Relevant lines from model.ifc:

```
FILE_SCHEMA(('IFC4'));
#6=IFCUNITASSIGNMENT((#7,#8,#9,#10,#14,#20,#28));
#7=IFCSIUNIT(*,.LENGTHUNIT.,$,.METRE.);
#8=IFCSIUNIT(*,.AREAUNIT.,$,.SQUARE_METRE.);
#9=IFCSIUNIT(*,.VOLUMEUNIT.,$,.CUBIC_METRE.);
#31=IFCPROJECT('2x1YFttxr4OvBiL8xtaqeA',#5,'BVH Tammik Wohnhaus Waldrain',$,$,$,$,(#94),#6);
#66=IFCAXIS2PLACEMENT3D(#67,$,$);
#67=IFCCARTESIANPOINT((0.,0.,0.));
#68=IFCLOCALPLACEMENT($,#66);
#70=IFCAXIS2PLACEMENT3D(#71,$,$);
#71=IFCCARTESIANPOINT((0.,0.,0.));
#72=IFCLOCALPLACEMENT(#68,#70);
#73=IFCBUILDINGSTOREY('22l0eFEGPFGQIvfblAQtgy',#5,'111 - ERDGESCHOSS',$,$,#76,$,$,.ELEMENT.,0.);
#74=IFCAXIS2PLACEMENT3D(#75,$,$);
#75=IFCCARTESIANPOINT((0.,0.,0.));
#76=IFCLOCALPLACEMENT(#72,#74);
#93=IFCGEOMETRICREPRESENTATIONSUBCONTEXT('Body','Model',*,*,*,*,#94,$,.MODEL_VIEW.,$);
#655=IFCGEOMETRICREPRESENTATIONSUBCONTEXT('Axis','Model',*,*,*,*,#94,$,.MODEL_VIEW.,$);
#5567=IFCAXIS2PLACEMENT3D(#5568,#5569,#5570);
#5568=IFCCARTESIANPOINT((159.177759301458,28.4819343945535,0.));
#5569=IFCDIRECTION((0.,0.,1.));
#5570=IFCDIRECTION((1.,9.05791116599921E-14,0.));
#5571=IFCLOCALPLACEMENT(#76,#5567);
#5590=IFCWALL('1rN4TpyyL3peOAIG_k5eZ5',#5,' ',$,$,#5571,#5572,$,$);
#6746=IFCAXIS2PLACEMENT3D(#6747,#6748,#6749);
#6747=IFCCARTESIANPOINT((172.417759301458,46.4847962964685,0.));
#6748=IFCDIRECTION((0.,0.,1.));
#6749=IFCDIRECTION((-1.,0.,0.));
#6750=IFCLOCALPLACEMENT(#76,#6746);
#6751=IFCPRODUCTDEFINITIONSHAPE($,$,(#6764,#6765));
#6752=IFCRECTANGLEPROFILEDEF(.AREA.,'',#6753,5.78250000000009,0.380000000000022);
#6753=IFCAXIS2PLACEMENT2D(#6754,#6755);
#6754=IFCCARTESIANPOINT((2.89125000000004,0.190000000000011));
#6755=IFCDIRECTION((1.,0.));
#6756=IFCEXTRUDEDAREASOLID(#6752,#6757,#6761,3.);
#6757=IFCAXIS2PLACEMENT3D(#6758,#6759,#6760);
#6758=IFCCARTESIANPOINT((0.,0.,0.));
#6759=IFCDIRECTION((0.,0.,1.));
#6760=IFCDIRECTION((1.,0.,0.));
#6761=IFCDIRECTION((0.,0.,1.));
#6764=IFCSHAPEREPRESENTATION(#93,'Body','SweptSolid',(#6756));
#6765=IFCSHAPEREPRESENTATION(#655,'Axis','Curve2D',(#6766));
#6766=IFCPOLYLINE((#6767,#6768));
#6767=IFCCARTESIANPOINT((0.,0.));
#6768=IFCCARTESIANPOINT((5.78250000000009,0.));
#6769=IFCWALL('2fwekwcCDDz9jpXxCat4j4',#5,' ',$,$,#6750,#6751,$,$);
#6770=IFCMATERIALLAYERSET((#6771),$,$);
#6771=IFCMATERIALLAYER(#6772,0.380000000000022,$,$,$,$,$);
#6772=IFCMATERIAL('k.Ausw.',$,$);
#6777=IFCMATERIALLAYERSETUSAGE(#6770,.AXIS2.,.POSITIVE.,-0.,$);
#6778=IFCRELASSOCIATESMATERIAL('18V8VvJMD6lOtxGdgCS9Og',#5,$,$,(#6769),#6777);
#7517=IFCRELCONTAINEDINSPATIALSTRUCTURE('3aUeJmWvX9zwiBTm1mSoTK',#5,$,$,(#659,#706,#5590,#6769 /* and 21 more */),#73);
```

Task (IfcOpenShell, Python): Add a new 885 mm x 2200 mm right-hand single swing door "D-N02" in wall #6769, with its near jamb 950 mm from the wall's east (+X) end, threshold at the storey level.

```python
import numpy as np
import ifcopenshell
import ifcopenshell.api.feature
import ifcopenshell.api.geometry
import ifcopenshell.api.root
import ifcopenshell.api.spatial
import ifcopenshell.geom
import ifcopenshell.util.element
import ifcopenshell.util.placement
import ifcopenshell.util.representation
import ifcopenshell.util.shape
import ifcopenshell.util.unit

model = ifcopenshell.open("model.ifc")
unit_scale = ifcopenshell.util.unit.calculate_unit_scale(model)
settings = ifcopenshell.geom.settings()


def volume(element):
    """Net volume in cubic metres, openings subtracted."""
    shape = ifcopenshell.geom.create_shape(settings, element)
    return ifcopenshell.util.shape.get_volume(shape.geometry)


wall = model.by_id(6769)
storey = ifcopenshell.util.element.get_container(wall, ifc_class="IfcBuildingStorey")
context = ifcopenshell.util.representation.get_context(model, "Model", "Body", "MODEL_VIEW")
before = volume(wall)

width, height, from_end, sill = 0.885, 2.2, 0.95, 0.0  # metres

# The wall runs along its own X axis, and the end named is its -X end.
wall_shape = ifcopenshell.geom.create_shape(settings, wall)
x, y, z = ifcopenshell.util.shape.get_vertices(wall_shape.geometry).T
start = x.min() + from_end
face, thickness = float(y.min()), float(y.max() - y.min())
wall_matrix = ifcopenshell.util.placement.get_local_placement(wall.ObjectPlacement)
level = ifcopenshell.util.placement.get_local_placement(storey.ObjectPlacement)[2, 3]


def in_wall(x, y):
    """Placement at x, y metres in the wall's axes, at sill height."""
    matrix = wall_matrix.copy()
    matrix[:, 3] = wall_matrix @ np.array([x / unit_scale, y / unit_scale, 0.0, 1.0])
    matrix[2, 3] = level + sill / unit_scale
    return matrix


# Opening: a box that overshoots both wall faces by 50 mm.
opening = ifcopenshell.api.root.create_entity(model, ifc_class="IfcOpeningElement", predefined_type="OPENING")
box = ifcopenshell.api.geometry.add_wall_representation(
    model, context=context, length=width, height=height, thickness=thickness + 0.1
)
ifcopenshell.api.geometry.assign_representation(model, product=opening, representation=box)
ifcopenshell.api.geometry.edit_object_placement(model, product=opening, matrix=in_wall(start, face - 0.05), is_si=False)
ifcopenshell.api.feature.add_feature(model, feature=opening, element=wall)

door = ifcopenshell.api.root.create_entity(model, ifc_class="IfcDoor", name="D-N02", predefined_type="DOOR")
door.OverallWidth, door.OverallHeight = width / unit_scale, height / unit_scale
door.OperationType = "SINGLE_SWING_RIGHT"
body = ifcopenshell.api.geometry.add_door_representation(
    model,
    context=context,
    overall_width=door.OverallWidth,
    overall_height=door.OverallHeight,
    operation_type="SINGLE_SWING_RIGHT",
    lining_properties={"LiningDepth": thickness / unit_scale, "ThresholdDepth": thickness / unit_scale},
)
ifcopenshell.api.geometry.assign_representation(model, product=door, representation=body)
ifcopenshell.api.spatial.assign_container(model, products=[door], relating_structure=storey)
ifcopenshell.api.feature.add_filling(model, opening=opening, element=door)

# The lining spans the wall, so the door starts at the wall face.
ifcopenshell.api.geometry.edit_object_placement(model, product=door, matrix=in_wall(start, face), is_si=False)

after = volume(wall)

print(f"wall volume {before:.3f} -> {after:.3f} m3")

model.write("model_v2.ifc")
```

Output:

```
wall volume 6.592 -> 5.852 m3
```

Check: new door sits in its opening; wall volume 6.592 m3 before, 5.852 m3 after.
